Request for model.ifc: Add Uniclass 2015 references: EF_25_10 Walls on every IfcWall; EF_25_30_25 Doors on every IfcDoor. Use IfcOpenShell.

First a look at what the model holds.

```python
import ifcopenshell

model = ifcopenshell.open("model.ifc")
print(model.schema)
print("classifications:", [c.Name for c in model.by_type("IfcClassification")])
for ifc_class in ("IfcDoor", "IfcRoof", "IfcStair", "IfcWall", "IfcWindow"):
    print(ifc_class, len(model.by_type(ifc_class)))
```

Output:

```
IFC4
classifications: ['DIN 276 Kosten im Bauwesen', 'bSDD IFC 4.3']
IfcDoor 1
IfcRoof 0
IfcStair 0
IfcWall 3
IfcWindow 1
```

```python
import ifcopenshell
import ifcopenshell.api.classification

model = ifcopenshell.open("model.ifc")

system = ifcopenshell.api.classification.add_classification(model, classification="Uniclass 2015")

codes = {
    "IfcWall": ("EF_25_10", "Walls"),
    "IfcDoor": ("EF_25_30_25", "Doors"),
}
for ifc_class, (code, name) in codes.items():
    products = model.by_type(ifc_class)
    ifcopenshell.api.classification.add_reference(
        model, products=products, classification=system, identification=code, name=name
    )
    print(code, len(products))

model.write("model_rev.ifc")
```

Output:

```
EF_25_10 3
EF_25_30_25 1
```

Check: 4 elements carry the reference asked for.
